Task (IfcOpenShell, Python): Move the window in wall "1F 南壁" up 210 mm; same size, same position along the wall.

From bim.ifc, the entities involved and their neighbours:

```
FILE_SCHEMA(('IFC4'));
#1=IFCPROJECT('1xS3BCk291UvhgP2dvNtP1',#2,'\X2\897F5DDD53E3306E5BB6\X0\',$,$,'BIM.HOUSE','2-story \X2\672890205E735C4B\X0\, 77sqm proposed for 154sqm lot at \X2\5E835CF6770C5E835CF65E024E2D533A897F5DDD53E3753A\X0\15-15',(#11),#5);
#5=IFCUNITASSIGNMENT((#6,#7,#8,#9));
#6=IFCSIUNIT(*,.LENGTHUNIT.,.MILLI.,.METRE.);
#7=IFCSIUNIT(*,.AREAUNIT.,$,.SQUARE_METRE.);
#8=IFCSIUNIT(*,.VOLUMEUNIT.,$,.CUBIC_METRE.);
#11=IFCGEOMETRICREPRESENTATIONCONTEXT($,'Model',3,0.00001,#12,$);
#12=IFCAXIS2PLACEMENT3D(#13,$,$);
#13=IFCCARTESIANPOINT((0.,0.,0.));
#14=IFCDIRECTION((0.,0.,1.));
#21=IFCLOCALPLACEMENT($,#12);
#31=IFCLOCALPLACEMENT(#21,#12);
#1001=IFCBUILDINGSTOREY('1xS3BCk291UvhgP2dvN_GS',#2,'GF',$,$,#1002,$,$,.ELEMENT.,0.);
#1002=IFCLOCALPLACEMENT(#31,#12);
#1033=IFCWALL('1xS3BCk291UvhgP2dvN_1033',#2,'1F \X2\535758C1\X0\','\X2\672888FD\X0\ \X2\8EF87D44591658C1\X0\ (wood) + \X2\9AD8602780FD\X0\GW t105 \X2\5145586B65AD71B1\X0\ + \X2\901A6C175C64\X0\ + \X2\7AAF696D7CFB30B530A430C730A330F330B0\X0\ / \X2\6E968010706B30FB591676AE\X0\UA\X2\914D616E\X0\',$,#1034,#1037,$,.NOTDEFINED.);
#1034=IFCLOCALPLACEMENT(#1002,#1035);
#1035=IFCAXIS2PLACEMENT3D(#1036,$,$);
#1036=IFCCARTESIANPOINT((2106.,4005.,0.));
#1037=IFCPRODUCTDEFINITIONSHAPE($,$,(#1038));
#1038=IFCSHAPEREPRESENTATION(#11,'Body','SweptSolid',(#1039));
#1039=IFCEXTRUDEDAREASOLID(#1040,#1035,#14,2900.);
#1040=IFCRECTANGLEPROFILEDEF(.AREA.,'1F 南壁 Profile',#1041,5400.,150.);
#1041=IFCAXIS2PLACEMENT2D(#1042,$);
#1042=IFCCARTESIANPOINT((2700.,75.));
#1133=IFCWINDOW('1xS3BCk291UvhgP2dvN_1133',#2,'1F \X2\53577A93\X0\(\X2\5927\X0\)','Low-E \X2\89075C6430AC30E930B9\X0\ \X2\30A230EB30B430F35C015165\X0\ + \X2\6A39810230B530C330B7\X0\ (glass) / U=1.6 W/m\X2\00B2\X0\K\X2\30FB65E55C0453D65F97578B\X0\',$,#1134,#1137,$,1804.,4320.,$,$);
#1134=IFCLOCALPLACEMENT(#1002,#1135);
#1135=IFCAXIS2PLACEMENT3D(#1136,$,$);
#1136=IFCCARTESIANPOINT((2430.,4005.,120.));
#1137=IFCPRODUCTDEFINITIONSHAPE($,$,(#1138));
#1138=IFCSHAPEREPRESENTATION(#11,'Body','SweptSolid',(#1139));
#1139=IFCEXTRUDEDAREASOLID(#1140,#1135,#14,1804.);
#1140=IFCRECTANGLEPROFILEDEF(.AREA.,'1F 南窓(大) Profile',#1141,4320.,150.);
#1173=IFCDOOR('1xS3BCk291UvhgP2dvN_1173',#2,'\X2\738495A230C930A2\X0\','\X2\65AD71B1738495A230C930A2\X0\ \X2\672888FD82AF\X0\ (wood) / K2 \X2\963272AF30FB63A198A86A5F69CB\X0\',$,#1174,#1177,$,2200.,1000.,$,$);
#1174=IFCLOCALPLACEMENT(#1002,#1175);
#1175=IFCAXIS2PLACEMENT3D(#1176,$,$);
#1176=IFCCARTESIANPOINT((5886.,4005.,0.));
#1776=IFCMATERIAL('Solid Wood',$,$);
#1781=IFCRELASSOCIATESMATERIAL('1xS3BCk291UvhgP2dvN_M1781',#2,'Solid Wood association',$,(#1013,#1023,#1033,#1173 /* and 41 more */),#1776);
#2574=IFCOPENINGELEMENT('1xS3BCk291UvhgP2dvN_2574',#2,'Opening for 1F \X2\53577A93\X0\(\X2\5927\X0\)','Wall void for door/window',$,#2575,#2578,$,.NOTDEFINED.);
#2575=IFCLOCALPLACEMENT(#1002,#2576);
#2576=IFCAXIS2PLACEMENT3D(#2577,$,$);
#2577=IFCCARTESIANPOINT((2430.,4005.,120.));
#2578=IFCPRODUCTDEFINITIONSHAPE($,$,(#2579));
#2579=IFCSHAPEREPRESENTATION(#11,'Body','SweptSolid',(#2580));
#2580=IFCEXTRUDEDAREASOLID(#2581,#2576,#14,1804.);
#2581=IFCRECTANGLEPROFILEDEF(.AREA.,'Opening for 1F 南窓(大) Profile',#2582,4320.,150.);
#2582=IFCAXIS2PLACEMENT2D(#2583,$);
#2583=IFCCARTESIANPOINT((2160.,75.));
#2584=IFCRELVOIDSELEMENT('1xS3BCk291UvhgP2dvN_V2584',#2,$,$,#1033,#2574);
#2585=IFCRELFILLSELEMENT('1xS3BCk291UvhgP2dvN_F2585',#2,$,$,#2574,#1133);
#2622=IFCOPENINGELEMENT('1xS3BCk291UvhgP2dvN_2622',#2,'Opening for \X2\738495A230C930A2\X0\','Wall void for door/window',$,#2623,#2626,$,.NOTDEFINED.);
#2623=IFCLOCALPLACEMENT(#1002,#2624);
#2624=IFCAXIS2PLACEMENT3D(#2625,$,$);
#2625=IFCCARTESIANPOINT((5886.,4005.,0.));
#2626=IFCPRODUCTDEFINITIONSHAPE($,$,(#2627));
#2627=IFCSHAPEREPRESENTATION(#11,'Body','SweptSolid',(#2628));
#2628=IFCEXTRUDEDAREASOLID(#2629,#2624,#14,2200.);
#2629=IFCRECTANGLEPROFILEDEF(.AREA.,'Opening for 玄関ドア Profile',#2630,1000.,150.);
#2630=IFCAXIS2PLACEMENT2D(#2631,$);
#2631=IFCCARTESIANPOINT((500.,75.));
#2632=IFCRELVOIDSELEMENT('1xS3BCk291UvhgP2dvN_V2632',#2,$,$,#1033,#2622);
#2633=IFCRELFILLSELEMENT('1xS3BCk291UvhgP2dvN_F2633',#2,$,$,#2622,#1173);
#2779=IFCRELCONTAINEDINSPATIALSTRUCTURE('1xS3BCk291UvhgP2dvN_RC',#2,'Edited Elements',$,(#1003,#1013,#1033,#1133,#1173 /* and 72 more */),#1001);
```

```python
import numpy as np
import ifcopenshell
import ifcopenshell.api.geometry
import ifcopenshell.util.placement
import ifcopenshell.util.unit

model = ifcopenshell.open("bim.ifc")
unit_scale = ifcopenshell.util.unit.calculate_unit_scale(model)

window = model.by_guid("1xS3BCk291UvhgP2dvN_1133")
opening = window.FillsVoids[0].RelatingOpeningElement
dz = 0.21 / unit_scale

shift = np.array([0.0, 0.0, dz])
# The window is not placed relative to its opening, so move both.
for product in (opening, window):
    matrix = ifcopenshell.util.placement.get_local_placement(product.ObjectPlacement)
    matrix[:3, 3] += shift
    ifcopenshell.api.geometry.edit_object_placement(model, product=product, matrix=matrix, is_si=False)

print(f"moved by {dz * unit_scale:+.3f} m")

model.write("bim_edited.ifc")
```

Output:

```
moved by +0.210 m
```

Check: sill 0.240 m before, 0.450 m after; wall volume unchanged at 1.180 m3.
